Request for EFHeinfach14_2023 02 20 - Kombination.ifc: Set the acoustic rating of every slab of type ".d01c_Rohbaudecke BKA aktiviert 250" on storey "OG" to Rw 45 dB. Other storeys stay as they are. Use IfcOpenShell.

First a look at what the model holds.

```python
import ifcopenshell
import ifcopenshell.util.element

model = ifcopenshell.open("EFHeinfach14_2023 02 20 - Kombination.ifc")
print(model.schema)
storey = next(s for s in model.by_type("IfcBuildingStorey") if s.Name == "OG")
slabs = [e for e in ifcopenshell.util.element.get_decomposition(storey) if e.is_a("IfcSlab")]
seen = {}
for e in slabs:
    element_type = ifcopenshell.util.element.get_type(e)
    key = (element_type.Name if element_type != e and element_type else None, ifcopenshell.util.element.get_pset(e, "Pset_SlabCommon", "AcousticRating"))
    seen[key] = seen.get(key, 0) + 1
for (name, value), count in sorted(seen.items(), key=str):
    print(count, "x", name, "|", value)
```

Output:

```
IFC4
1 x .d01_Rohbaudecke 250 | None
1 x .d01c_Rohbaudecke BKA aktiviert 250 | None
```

```python
import ifcopenshell
import ifcopenshell.api.pset
import ifcopenshell.util.element

model = ifcopenshell.open("EFHeinfach14_2023 02 20 - Kombination.ifc")

storey = next(s for s in model.by_type("IfcBuildingStorey") if s.Name == "OG")
slabs = [e for e in ifcopenshell.util.element.get_decomposition(storey) if e.is_a("IfcSlab")]

count = 0
for e in slabs:
    element_type = ifcopenshell.util.element.get_type(e)
    if element_type in (None, e) or element_type.Name != ".d01c_Rohbaudecke BKA aktiviert 250":
        continue
    # add_pset returns the element's existing set when there is one.
    pset = ifcopenshell.api.pset.add_pset(model, product=e, name="Pset_SlabCommon")
    ifcopenshell.api.pset.edit_pset(model, pset=pset, properties={"AcousticRating": "Rw 45 dB"})
    count += 1

print(count, "slabs updated")

model.write("EFHeinfach14_2023 02 20 - Kombination-out.ifc")
```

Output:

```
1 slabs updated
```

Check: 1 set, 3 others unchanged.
